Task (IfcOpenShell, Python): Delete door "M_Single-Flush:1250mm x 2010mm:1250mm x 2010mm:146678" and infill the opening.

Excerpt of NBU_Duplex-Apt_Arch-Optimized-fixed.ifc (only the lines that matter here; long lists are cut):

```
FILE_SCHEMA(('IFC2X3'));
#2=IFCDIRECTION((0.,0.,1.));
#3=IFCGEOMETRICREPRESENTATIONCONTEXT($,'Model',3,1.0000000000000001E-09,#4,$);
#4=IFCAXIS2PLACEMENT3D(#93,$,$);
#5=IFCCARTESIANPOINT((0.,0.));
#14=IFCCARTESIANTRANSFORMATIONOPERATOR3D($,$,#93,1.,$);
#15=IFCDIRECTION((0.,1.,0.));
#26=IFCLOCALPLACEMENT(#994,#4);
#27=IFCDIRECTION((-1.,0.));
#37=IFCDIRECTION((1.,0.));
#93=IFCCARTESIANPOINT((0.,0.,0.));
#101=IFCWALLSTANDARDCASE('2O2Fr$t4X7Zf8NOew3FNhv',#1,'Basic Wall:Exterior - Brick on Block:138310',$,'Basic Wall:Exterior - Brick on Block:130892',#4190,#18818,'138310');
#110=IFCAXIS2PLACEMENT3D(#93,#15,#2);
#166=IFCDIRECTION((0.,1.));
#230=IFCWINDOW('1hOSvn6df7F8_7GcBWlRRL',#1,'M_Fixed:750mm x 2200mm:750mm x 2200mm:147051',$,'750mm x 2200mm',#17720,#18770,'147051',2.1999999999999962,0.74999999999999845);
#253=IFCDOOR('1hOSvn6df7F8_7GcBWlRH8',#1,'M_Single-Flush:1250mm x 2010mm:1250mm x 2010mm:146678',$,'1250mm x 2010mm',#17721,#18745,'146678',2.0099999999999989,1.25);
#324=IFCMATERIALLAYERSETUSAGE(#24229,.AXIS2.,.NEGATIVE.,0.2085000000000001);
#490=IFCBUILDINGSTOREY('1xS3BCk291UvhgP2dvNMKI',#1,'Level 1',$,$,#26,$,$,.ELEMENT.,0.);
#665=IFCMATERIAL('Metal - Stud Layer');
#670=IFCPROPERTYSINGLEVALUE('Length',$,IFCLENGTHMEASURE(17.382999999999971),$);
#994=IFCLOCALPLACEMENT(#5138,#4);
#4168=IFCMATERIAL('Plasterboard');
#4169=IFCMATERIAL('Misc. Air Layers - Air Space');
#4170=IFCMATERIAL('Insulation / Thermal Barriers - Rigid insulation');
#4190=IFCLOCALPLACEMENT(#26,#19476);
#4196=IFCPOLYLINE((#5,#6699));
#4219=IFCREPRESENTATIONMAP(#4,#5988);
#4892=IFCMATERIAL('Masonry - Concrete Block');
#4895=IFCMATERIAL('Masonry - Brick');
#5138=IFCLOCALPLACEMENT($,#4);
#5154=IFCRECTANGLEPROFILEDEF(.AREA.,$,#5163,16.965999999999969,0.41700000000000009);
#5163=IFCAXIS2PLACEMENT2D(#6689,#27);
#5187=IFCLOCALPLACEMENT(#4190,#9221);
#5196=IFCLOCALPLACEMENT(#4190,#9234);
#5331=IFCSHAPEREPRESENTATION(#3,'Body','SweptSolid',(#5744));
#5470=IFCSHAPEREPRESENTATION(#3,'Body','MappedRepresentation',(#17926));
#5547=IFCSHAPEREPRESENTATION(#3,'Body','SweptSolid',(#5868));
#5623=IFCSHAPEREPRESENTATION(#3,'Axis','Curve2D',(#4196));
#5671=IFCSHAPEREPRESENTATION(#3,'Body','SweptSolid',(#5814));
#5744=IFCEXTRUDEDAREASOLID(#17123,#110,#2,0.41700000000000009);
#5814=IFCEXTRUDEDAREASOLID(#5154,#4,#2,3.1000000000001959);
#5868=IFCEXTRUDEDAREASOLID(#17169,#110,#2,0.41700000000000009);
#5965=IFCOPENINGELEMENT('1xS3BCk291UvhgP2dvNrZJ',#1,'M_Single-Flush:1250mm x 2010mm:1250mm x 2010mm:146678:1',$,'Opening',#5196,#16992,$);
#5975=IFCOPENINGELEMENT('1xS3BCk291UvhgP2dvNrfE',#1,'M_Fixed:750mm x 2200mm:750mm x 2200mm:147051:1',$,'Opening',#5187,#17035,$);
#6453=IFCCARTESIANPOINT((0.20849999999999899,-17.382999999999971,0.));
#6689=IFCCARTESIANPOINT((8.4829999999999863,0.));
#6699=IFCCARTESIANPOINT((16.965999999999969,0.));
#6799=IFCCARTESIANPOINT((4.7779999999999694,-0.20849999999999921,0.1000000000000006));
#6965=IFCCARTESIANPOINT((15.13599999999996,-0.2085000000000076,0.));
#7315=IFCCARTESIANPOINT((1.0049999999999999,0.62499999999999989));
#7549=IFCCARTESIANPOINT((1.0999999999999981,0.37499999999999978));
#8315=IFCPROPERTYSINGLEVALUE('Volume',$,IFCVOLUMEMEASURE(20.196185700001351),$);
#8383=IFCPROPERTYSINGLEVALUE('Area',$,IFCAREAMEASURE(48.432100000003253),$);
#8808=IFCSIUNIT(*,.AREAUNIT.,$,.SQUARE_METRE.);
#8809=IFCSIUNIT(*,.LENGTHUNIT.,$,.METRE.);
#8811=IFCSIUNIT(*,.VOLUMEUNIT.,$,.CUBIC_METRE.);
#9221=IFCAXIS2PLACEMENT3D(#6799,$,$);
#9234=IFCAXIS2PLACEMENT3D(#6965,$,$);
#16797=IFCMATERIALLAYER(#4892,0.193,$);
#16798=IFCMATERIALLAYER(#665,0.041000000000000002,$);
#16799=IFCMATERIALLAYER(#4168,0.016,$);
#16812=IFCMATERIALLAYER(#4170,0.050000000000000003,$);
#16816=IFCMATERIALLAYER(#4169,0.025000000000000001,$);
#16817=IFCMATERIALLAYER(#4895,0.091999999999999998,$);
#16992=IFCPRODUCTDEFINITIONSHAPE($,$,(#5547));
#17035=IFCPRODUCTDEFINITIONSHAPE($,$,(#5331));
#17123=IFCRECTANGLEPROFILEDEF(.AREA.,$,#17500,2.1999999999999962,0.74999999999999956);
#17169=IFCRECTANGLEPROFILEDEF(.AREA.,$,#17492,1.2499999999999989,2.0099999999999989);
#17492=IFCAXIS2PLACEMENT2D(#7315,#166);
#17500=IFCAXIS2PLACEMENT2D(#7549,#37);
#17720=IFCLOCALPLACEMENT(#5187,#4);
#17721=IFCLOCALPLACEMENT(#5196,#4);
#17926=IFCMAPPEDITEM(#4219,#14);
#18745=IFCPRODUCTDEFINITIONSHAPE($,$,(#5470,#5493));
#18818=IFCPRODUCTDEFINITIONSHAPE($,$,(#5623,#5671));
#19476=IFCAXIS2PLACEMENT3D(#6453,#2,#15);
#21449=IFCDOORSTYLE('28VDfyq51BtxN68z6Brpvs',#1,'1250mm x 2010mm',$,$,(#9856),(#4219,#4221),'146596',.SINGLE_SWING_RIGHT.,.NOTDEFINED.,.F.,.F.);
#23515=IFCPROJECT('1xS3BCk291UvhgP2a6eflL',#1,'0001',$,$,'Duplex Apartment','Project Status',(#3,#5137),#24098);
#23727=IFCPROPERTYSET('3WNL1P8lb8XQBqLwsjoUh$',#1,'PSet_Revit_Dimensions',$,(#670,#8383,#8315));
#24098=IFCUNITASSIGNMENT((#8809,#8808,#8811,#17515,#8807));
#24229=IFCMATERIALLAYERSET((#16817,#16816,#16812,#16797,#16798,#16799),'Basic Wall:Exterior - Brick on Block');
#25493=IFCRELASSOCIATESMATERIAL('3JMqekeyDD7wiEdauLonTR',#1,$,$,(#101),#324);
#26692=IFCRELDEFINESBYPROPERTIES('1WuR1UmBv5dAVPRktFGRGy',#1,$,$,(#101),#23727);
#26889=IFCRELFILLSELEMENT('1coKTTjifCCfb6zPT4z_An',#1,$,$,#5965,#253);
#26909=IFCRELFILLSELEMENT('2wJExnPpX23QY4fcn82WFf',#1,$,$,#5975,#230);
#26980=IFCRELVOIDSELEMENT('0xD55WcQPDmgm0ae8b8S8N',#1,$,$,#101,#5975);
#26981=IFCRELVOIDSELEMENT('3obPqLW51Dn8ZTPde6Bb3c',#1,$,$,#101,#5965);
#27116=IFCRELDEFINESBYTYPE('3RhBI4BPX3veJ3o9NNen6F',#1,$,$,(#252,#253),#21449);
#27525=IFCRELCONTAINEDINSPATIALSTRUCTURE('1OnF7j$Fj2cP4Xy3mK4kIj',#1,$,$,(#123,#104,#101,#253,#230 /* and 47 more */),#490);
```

```python
import ifcopenshell
import ifcopenshell.api.feature
import ifcopenshell.api.pset
import ifcopenshell.api.root
import ifcopenshell.geom
import ifcopenshell.util.element
import ifcopenshell.util.shape
import ifcopenshell.util.unit

model = ifcopenshell.open("NBU_Duplex-Apt_Arch-Optimized-fixed.ifc")
area_scale = ifcopenshell.util.unit.calculate_unit_scale(model, "AREAUNIT")
volume_scale = ifcopenshell.util.unit.calculate_unit_scale(model, "VOLUMEUNIT")
settings = ifcopenshell.geom.settings()


def volume(element):
    """Net volume in cubic metres, openings subtracted."""
    shape = ifcopenshell.geom.create_shape(settings, element)
    return ifcopenshell.util.shape.get_volume(shape.geometry)


door = model.by_guid("1hOSvn6df7F8_7GcBWlRH8")
opening = door.FillsVoids[0].RelatingOpeningElement
wall = opening.VoidsElements[0].RelatingBuildingElement
before = volume(wall)

ifcopenshell.api.root.remove_product(model, product=door)
ifcopenshell.api.feature.remove_feature(model, feature=opening)

after = volume(wall)
thickness = 0.417  # wall thickness in metres

# Update the wall's stored quantities.
pset = model.by_id(ifcopenshell.util.element.get_pset(wall, "PSet_Revit_Dimensions", should_inherit=False)["id"])
ifcopenshell.api.pset.edit_pset(model, pset=pset, properties={
    "Area": model.create_entity("IfcAreaMeasure", after / thickness / area_scale),
    "Volume": model.create_entity("IfcVolumeMeasure", after / volume_scale),
})

print(f"wall volume {before:.3f} -> {after:.3f} m3")

model.write("NBU_Duplex-Apt_Arch-Optimized-fixed_rev.ifc")
```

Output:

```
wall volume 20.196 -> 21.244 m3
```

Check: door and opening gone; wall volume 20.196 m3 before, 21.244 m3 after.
